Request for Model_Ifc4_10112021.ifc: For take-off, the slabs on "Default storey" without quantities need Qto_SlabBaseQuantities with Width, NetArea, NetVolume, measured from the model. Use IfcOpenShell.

First a look at what the model holds.

```python
import ifcopenshell
import ifcopenshell.util.element
import ifcopenshell.util.unit

model = ifcopenshell.open("Model_Ifc4_10112021.ifc")
print(model.schema)
for unit_type in ("LENGTHUNIT", "AREAUNIT", "VOLUMEUNIT"):
    print(unit_type, ifcopenshell.util.unit.calculate_unit_scale(model, unit_type))
storey = next(s for s in model.by_type("IfcBuildingStorey") if s.Name == "Default storey")
slabs = [e for e in ifcopenshell.util.element.get_decomposition(storey) if e.is_a("IfcSlab")]
for e in sorted(slabs, key=lambda e: e.id()):
    print(e.id(), e.is_a(), e.Name, list(ifcopenshell.util.element.get_psets(e, qtos_only=True)), sep=" | ")
```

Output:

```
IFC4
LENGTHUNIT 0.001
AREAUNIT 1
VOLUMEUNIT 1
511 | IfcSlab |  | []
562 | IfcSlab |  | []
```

```python
import ifcopenshell
import ifcopenshell.api.pset
import ifcopenshell.geom
import ifcopenshell.util.element
import ifcopenshell.util.shape
import ifcopenshell.util.unit

model = ifcopenshell.open("Model_Ifc4_10112021.ifc")
unit_scale = ifcopenshell.util.unit.calculate_unit_scale(model)
area_scale = ifcopenshell.util.unit.calculate_unit_scale(model, "AREAUNIT")
volume_scale = ifcopenshell.util.unit.calculate_unit_scale(model, "VOLUMEUNIT")
settings = ifcopenshell.geom.settings()

storey = next(s for s in model.by_type("IfcBuildingStorey") if s.Name == "Default storey")
slabs = [e for e in ifcopenshell.util.element.get_decomposition(storey) if e.is_a("IfcSlab")]

for e in sorted(slabs, key=lambda e: e.id()):
    if ifcopenshell.util.element.get_psets(e, qtos_only=True, should_inherit=False):
        continue
    # Geometry comes back in metres, in the element's own axes.
    shape = ifcopenshell.geom.create_shape(settings, e)
    values = {
        "Width": ifcopenshell.util.shape.get_z(shape.geometry) / unit_scale,
        "NetArea": ifcopenshell.util.shape.get_footprint_area(shape.geometry) / area_scale,
        "NetVolume": ifcopenshell.util.shape.get_volume(shape.geometry) / volume_scale,
    }
    qto = ifcopenshell.api.pset.add_qto(model, product=e, name="Qto_SlabBaseQuantities")
    ifcopenshell.api.pset.edit_qto(model, qto=qto, properties=values)
    print(e.id(), {k: round(v, 3) for k, v in values.items()})

model.write("Model_Ifc4_10112021-out.ifc")
```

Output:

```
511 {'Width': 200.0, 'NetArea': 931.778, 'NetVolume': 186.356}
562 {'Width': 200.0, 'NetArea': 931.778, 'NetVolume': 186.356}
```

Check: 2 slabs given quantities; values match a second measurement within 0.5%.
